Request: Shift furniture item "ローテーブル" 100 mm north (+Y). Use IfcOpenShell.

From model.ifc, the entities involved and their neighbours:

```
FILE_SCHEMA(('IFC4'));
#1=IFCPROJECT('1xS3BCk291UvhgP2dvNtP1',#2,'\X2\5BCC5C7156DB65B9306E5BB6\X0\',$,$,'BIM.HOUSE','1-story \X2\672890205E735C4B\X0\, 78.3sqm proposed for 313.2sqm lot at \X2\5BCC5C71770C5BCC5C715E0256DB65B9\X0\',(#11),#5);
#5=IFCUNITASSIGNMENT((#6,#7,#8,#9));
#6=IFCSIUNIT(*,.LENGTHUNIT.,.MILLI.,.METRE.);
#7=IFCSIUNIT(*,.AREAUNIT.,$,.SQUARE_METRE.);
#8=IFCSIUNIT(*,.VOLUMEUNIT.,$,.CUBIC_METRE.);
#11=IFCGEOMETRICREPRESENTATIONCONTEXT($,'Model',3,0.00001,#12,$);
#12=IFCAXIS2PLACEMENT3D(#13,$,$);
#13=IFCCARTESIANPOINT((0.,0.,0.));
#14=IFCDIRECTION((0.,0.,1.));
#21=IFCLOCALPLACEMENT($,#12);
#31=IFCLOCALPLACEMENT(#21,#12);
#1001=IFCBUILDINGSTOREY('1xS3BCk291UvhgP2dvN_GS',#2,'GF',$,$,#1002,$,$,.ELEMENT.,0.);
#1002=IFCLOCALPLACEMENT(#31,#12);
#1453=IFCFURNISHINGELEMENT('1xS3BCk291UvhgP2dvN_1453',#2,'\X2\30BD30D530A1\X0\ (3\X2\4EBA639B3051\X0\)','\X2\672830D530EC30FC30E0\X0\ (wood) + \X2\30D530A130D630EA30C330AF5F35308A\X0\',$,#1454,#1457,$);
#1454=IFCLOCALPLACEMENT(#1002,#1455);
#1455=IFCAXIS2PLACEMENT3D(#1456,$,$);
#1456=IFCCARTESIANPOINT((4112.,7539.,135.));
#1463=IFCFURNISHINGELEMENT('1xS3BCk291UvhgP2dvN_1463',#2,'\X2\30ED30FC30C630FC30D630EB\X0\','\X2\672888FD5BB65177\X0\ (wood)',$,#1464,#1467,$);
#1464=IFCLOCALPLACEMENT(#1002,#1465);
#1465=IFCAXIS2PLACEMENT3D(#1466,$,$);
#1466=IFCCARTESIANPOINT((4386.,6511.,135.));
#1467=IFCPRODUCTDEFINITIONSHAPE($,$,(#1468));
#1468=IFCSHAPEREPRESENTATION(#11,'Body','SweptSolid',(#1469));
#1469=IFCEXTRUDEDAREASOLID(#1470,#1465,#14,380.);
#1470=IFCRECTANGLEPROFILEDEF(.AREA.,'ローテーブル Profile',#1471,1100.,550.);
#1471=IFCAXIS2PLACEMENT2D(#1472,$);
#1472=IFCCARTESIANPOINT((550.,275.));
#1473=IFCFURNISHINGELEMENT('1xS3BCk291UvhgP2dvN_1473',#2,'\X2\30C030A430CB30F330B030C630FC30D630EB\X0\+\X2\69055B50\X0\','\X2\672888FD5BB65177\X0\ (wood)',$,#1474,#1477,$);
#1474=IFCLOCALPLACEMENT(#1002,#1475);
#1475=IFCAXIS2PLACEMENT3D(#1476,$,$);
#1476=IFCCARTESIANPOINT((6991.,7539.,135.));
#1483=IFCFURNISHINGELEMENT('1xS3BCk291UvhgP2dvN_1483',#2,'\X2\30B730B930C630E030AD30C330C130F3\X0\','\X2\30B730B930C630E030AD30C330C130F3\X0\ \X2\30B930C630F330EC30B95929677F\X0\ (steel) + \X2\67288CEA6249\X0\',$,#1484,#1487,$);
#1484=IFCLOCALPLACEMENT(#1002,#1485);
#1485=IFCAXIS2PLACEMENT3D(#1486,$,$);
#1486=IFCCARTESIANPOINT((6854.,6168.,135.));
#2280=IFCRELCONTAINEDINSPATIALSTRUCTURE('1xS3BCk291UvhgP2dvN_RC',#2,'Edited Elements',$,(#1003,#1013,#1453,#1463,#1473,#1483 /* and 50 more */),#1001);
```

```python
import ifcopenshell
import ifcopenshell.api.geometry
import ifcopenshell.util.placement

model = ifcopenshell.open("model.ifc")

item = model.by_guid("1xS3BCk291UvhgP2dvN_1463")
matrix = ifcopenshell.util.placement.get_local_placement(item.ObjectPlacement)
matrix[1, 3] += 100.0
ifcopenshell.api.geometry.edit_object_placement(model, product=item, matrix=matrix, is_si=False)

print(ifcopenshell.util.placement.get_local_placement(item.ObjectPlacement).round(3) + 0.0)

model.write("model_updated.ifc")
```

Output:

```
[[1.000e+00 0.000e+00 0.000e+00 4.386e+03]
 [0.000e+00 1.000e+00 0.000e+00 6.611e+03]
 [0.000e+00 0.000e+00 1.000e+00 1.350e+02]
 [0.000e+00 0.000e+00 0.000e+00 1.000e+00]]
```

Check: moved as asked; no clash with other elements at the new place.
